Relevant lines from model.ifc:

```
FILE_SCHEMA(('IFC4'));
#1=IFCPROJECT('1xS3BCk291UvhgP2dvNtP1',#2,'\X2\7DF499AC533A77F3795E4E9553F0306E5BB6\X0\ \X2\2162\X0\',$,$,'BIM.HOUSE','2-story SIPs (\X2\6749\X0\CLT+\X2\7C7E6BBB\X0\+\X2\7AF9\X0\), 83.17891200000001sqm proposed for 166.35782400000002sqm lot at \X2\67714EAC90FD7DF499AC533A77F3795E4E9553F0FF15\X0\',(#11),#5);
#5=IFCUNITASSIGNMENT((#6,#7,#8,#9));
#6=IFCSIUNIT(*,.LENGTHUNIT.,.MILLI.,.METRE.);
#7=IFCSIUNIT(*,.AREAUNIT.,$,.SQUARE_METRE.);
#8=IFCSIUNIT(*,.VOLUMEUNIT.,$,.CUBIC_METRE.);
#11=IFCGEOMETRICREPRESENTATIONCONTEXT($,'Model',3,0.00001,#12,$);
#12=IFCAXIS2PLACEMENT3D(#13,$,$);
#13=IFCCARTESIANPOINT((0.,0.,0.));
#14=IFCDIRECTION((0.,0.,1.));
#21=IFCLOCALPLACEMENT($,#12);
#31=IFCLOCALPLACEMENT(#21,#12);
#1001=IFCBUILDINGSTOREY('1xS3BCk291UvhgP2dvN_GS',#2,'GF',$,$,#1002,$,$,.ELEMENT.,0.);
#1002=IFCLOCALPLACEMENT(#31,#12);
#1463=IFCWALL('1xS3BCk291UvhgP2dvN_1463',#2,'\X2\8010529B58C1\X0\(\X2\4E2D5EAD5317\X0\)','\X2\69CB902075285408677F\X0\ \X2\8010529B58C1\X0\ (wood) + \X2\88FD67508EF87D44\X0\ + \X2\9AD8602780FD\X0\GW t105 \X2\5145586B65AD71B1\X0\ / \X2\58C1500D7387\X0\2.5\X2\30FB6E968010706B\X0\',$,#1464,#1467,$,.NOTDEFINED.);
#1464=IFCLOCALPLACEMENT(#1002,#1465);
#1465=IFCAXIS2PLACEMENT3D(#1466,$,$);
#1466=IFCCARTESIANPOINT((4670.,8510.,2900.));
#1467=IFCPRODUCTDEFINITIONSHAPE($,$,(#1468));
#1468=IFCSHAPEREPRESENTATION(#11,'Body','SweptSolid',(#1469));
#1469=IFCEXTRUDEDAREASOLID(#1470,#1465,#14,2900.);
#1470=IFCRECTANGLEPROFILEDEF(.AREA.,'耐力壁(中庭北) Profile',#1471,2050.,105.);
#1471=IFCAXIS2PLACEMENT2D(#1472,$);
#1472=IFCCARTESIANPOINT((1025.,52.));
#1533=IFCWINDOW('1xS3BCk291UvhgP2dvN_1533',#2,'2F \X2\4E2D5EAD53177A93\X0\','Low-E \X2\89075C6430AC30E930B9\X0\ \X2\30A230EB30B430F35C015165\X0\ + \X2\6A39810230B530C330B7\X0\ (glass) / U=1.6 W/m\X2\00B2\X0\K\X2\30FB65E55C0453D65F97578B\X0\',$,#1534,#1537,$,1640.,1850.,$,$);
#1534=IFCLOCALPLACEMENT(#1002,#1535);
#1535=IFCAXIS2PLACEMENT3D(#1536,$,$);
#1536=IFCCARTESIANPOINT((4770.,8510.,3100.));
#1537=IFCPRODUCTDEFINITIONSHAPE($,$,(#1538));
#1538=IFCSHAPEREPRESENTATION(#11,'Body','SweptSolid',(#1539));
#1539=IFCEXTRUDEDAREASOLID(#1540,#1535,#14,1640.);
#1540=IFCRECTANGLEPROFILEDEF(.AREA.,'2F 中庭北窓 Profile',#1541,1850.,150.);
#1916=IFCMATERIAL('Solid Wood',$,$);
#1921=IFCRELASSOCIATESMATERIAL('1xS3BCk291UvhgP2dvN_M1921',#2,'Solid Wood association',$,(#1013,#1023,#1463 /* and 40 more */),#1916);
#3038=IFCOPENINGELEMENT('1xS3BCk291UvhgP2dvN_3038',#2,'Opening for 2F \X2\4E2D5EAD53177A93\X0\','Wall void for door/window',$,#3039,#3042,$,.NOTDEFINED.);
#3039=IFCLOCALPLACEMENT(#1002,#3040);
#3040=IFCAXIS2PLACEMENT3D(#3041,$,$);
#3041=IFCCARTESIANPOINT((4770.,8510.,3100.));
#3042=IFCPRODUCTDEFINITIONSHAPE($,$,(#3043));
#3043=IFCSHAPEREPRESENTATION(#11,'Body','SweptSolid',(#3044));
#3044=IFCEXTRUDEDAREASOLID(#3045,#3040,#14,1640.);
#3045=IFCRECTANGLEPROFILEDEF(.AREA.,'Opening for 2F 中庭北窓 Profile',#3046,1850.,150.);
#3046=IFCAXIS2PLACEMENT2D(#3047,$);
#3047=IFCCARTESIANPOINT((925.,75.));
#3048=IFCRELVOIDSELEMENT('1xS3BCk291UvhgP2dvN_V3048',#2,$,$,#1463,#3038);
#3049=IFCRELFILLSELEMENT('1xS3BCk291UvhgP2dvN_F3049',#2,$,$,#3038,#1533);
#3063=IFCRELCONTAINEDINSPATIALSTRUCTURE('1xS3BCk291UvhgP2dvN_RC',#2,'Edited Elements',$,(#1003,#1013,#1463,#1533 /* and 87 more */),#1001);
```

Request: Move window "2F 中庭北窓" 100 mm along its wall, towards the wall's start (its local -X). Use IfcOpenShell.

```python
import ifcopenshell
import ifcopenshell.api.geometry
import ifcopenshell.util.placement
import ifcopenshell.util.unit

model = ifcopenshell.open("model.ifc")
unit_scale = ifcopenshell.util.unit.calculate_unit_scale(model)

window = model.by_id(1533)
opening = window.FillsVoids[0].RelatingOpeningElement
wall = opening.VoidsElements[0].RelatingBuildingElement

wall_matrix = ifcopenshell.util.placement.get_local_placement(wall.ObjectPlacement)
shift = wall_matrix[:3, 0] * -0.1 / unit_scale
before = ifcopenshell.util.placement.get_local_placement(window.ObjectPlacement)[:3, 3].copy()

# The window is not placed relative to its opening, so move both.
for product in (opening, window):
    matrix = ifcopenshell.util.placement.get_local_placement(product.ObjectPlacement)
    matrix[:3, 3] += shift
    ifcopenshell.api.geometry.edit_object_placement(model, product=product, matrix=matrix, is_si=False)

after = ifcopenshell.util.placement.get_local_placement(window.ObjectPlacement)[:3, 3]
print("window moved by", (after - before).round(3) + 0.0)

model.write("model-out.ifc")
```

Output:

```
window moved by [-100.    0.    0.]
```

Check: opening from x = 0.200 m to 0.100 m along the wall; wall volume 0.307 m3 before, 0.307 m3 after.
